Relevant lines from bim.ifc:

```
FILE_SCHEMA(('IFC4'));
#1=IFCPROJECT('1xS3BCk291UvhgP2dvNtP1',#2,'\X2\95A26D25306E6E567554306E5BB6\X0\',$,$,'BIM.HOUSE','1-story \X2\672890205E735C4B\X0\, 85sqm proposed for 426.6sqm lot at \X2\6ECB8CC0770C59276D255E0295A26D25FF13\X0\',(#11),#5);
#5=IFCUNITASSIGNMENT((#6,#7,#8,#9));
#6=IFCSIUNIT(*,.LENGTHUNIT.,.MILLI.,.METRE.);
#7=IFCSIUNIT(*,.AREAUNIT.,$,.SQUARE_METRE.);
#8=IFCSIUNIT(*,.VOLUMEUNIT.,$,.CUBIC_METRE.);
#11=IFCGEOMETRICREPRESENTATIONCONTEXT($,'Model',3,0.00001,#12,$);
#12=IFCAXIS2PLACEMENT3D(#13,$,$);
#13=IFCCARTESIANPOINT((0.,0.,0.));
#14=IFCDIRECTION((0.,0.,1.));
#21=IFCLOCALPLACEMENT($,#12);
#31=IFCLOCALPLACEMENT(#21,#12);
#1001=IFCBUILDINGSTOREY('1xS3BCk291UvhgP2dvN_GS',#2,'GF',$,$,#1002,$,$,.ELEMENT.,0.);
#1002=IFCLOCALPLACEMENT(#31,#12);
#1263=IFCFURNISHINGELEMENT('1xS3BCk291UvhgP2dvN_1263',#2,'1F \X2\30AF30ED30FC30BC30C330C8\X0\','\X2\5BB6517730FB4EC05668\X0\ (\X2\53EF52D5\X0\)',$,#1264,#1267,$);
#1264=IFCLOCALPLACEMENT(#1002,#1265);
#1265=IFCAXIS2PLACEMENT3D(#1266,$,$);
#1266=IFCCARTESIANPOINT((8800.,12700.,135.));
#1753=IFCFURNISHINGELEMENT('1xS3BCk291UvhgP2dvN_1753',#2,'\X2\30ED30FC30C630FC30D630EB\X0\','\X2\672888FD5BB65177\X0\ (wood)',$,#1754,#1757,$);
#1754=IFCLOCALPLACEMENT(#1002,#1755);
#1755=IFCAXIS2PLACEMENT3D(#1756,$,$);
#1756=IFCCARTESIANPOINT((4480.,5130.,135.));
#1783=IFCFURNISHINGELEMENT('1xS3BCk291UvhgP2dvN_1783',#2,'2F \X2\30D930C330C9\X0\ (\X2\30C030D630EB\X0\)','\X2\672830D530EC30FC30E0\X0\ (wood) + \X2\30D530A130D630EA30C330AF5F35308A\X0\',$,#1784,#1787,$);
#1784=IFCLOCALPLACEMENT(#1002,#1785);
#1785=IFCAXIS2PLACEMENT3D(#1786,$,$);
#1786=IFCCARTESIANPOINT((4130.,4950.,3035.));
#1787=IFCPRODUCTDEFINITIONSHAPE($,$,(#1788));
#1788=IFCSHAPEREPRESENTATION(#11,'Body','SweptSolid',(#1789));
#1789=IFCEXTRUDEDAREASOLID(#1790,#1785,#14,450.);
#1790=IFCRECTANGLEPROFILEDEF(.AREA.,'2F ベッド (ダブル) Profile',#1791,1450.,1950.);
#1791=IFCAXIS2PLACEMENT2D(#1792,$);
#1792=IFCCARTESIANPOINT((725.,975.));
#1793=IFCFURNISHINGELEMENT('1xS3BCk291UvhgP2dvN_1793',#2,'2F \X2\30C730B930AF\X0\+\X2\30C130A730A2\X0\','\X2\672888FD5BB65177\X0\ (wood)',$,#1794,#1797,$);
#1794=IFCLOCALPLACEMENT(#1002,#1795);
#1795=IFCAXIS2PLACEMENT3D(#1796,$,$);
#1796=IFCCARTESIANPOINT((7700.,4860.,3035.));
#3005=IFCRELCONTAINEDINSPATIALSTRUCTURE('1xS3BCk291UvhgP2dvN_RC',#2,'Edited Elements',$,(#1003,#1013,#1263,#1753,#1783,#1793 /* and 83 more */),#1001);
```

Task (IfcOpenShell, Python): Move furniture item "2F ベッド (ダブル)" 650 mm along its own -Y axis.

```python
import ifcopenshell
import ifcopenshell.api.geometry
import ifcopenshell.util.placement
import ifcopenshell.util.unit

model = ifcopenshell.open("bim.ifc")
unit_scale = ifcopenshell.util.unit.calculate_unit_scale(model)

item = model.by_id(1783)
matrix = ifcopenshell.util.placement.get_local_placement(item.ObjectPlacement)
matrix[:3, 3] -= matrix[:3, 1] * 0.65 / unit_scale
ifcopenshell.api.geometry.edit_object_placement(model, product=item, matrix=matrix, is_si=False)

print(ifcopenshell.util.placement.get_local_placement(item.ObjectPlacement).round(3) + 0.0)

model.write("bim_rev.ifc")
```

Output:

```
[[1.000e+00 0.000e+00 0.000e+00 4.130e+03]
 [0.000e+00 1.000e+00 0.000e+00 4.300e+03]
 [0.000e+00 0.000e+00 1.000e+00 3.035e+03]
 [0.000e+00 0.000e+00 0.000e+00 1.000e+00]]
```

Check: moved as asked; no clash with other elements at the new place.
